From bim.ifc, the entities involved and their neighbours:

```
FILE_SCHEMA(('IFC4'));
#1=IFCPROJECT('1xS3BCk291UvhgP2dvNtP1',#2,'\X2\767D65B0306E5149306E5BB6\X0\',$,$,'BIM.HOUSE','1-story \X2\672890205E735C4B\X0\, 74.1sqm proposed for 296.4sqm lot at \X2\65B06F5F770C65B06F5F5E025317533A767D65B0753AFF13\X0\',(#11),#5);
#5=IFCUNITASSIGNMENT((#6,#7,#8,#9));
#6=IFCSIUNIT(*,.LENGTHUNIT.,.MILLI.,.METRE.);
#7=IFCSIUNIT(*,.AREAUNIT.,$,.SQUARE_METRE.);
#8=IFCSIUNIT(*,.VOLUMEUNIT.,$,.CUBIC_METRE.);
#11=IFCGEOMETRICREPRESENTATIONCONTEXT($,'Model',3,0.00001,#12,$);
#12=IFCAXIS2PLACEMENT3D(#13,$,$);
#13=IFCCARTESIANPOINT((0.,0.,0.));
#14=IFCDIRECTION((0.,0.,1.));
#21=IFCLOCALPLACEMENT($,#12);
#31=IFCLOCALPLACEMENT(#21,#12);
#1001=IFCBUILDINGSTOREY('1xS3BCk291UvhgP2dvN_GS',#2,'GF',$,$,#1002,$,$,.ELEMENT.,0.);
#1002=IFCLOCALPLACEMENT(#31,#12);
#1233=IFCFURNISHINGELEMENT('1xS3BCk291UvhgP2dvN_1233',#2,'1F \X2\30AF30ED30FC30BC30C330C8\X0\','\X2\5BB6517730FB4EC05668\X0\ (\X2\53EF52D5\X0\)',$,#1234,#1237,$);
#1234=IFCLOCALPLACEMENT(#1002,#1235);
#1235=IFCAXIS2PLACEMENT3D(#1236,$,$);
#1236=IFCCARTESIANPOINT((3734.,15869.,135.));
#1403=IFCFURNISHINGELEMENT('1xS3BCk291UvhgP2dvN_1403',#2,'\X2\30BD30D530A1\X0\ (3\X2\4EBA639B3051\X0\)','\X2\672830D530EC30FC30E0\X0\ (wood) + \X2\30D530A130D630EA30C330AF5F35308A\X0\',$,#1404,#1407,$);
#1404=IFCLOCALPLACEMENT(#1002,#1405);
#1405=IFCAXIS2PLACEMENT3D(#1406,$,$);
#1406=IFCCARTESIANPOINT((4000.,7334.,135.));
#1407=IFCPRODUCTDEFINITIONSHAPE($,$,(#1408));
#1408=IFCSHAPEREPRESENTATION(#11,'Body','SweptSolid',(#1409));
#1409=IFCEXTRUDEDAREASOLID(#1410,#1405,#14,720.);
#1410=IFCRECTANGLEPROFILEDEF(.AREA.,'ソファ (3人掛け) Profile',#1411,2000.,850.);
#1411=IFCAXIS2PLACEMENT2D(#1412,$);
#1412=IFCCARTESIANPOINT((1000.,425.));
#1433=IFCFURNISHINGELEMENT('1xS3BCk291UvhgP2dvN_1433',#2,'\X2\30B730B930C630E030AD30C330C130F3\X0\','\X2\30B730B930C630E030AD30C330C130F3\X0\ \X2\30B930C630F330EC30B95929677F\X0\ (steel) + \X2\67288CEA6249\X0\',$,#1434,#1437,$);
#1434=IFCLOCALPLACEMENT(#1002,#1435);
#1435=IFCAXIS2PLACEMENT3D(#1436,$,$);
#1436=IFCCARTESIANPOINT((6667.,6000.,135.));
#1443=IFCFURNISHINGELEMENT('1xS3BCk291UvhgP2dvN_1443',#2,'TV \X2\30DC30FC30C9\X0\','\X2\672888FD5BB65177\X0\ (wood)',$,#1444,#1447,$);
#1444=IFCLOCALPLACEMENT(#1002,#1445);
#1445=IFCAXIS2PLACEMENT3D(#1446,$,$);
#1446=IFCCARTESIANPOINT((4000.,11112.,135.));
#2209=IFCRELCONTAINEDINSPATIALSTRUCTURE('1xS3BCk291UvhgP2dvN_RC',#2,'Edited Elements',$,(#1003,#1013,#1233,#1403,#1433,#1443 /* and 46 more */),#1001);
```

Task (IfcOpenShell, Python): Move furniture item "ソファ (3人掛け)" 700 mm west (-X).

```python
import ifcopenshell
import ifcopenshell.api.geometry
import ifcopenshell.util.placement
import ifcopenshell.util.unit

model = ifcopenshell.open("bim.ifc")
unit_scale = ifcopenshell.util.unit.calculate_unit_scale(model)

item = model.by_guid("1xS3BCk291UvhgP2dvN_1403")
matrix = ifcopenshell.util.placement.get_local_placement(item.ObjectPlacement)
matrix[0, 3] -= 0.7 / unit_scale
ifcopenshell.api.geometry.edit_object_placement(model, product=item, matrix=matrix, is_si=False)

print(ifcopenshell.util.placement.get_local_placement(item.ObjectPlacement).round(3) + 0.0)

model.write("bim_rev.ifc")
```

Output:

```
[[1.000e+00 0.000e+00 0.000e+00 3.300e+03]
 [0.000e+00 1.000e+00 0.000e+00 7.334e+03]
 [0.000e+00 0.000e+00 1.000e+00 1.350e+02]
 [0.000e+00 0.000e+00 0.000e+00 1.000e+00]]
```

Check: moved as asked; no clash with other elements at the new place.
